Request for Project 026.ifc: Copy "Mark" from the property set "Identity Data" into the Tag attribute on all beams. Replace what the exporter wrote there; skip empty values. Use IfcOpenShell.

First a look at what the model holds.

```python
import ifcopenshell
import ifcopenshell.util.element

model = ifcopenshell.open("Project 026.ifc")
print(model.schema)
beams = model.by_type("IfcBeam")
print(len(beams), "beams")
for e in beams[:8]:
    source = ifcopenshell.util.element.get_pset(e, "Identity Data", "Mark")
    target = e.Tag
    print(e.id(), repr(source), repr(target), sep=" | ")
```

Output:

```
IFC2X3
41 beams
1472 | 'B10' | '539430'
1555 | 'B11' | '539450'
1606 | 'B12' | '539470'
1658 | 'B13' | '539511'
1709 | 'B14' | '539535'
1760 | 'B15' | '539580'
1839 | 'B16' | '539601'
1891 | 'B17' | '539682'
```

```python
import ifcopenshell
import ifcopenshell.util.element

model = ifcopenshell.open("Project 026.ifc")

count = 0
for e in model.by_type("IfcBeam"):
    value = ifcopenshell.util.element.get_pset(e, "Identity Data", "Mark")
    current = e.Tag
    if not value or not value.strip() or current == value:
        continue
    e.Tag = value
    count += 1

print(count, "beams updated")

model.write("Project 026_updated.ifc")
```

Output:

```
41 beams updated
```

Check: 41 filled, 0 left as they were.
